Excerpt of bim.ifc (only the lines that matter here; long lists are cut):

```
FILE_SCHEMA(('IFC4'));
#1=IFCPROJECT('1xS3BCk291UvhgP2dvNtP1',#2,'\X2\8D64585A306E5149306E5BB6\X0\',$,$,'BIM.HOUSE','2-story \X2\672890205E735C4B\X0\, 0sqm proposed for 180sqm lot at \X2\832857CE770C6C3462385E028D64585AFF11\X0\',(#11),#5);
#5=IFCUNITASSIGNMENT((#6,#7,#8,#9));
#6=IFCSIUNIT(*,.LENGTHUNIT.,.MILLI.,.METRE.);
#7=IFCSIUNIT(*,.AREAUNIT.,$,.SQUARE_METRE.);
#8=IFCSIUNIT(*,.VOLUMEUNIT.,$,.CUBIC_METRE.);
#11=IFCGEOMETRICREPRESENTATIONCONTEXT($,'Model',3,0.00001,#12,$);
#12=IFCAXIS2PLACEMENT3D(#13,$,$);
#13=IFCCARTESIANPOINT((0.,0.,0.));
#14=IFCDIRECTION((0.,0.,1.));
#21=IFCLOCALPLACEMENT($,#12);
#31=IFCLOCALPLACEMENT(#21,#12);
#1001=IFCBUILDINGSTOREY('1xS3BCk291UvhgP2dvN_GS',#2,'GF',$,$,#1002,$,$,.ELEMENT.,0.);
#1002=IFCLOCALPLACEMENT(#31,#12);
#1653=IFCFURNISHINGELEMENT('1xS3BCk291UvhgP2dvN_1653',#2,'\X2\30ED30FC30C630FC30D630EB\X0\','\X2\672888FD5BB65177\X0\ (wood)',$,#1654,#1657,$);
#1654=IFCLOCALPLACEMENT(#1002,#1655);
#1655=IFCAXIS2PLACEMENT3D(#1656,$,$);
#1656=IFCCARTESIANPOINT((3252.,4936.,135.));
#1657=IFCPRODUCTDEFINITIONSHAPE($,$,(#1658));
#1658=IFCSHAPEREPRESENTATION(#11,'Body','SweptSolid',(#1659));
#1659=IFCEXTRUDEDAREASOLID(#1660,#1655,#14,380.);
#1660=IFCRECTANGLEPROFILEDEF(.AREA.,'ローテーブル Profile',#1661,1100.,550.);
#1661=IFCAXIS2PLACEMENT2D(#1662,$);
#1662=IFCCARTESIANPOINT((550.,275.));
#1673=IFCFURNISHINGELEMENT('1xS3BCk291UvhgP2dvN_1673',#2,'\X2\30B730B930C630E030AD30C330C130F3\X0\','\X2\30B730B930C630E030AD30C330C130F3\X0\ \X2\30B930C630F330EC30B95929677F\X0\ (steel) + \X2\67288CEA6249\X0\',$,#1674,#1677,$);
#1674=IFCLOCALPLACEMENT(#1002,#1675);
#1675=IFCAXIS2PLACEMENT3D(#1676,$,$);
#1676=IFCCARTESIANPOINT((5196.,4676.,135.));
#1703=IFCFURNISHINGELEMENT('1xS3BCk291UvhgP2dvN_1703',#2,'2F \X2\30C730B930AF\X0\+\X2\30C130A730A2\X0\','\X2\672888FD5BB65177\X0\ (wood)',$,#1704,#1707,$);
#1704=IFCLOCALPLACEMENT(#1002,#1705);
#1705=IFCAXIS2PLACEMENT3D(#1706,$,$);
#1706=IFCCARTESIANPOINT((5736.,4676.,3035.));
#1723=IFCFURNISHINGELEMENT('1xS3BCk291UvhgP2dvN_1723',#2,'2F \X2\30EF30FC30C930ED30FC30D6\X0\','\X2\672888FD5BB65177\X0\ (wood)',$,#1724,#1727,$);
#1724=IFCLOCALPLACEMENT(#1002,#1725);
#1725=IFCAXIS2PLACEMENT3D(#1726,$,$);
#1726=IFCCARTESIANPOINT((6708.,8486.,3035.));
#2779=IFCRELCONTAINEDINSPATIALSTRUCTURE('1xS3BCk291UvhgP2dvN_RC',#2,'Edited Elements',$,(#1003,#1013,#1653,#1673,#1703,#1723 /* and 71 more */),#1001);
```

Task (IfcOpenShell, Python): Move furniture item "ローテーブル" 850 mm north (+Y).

```python
import ifcopenshell
import ifcopenshell.api.geometry
import ifcopenshell.util.placement

model = ifcopenshell.open("bim.ifc")

item = model.by_guid("1xS3BCk291UvhgP2dvN_1653")
matrix = ifcopenshell.util.placement.get_local_placement(item.ObjectPlacement)
matrix[1, 3] += 850.0
ifcopenshell.api.geometry.edit_object_placement(model, product=item, matrix=matrix, is_si=False)

print(ifcopenshell.util.placement.get_local_placement(item.ObjectPlacement).round(3) + 0.0)

model.write("bim_updated.ifc")
```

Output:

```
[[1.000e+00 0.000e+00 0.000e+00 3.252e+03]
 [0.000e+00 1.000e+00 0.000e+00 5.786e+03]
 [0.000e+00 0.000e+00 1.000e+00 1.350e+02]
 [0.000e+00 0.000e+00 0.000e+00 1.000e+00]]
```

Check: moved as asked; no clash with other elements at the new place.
